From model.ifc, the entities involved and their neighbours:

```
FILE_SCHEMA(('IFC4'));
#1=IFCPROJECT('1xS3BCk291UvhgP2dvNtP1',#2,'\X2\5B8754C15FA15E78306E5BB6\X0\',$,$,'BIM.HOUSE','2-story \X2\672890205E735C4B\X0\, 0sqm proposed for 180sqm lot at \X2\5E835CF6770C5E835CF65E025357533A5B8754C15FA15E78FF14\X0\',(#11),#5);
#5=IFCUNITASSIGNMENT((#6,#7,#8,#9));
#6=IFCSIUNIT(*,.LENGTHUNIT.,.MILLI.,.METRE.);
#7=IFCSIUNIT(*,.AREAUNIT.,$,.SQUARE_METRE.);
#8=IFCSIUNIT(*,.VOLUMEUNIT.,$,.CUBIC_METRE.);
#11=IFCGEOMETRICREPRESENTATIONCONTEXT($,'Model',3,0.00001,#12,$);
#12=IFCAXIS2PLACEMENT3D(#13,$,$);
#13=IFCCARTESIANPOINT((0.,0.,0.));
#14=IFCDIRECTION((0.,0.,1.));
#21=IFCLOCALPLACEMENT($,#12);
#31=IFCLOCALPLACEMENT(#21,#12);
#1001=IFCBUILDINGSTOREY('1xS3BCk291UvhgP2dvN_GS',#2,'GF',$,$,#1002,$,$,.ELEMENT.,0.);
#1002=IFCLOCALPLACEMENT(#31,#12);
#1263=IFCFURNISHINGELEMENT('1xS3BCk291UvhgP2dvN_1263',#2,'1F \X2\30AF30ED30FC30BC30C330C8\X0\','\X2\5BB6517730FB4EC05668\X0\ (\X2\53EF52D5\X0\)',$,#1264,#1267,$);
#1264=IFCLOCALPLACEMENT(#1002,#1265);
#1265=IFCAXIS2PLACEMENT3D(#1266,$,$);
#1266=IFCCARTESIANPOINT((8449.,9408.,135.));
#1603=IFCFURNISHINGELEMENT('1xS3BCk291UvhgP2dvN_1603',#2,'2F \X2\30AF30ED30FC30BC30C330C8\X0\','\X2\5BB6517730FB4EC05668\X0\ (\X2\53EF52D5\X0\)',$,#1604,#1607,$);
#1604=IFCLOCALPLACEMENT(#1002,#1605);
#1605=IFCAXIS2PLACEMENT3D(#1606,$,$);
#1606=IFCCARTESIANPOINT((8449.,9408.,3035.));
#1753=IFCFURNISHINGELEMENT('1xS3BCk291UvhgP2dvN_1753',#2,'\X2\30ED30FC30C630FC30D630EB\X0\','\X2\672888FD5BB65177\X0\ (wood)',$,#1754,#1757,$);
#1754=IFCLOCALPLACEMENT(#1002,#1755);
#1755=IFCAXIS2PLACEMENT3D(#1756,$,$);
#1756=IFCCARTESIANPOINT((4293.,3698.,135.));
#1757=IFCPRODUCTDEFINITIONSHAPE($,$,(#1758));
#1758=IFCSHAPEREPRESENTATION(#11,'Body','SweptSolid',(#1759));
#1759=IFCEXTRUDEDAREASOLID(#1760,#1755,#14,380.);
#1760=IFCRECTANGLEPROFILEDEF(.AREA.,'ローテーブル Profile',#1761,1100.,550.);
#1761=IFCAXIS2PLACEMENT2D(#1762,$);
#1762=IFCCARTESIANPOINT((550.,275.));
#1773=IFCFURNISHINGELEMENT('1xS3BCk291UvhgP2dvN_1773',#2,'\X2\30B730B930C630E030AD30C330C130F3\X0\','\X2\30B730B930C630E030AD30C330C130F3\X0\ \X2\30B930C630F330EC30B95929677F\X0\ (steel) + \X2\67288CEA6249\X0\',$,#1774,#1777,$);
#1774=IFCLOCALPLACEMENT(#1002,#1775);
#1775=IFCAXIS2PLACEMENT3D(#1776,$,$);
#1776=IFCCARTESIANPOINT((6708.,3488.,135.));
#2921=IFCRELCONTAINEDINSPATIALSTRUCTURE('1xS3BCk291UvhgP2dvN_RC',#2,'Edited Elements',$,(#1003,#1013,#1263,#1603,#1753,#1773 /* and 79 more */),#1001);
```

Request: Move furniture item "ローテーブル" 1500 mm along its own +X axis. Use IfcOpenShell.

```python
import ifcopenshell
import ifcopenshell.api.geometry
import ifcopenshell.util.placement
import ifcopenshell.util.unit

model = ifcopenshell.open("model.ifc")
unit_scale = ifcopenshell.util.unit.calculate_unit_scale(model)

item = model.by_id(1753)
matrix = ifcopenshell.util.placement.get_local_placement(item.ObjectPlacement)
matrix[:3, 3] += matrix[:3, 0] * 1.5 / unit_scale
ifcopenshell.api.geometry.edit_object_placement(model, product=item, matrix=matrix, is_si=False)

print(ifcopenshell.util.placement.get_local_placement(item.ObjectPlacement).round(3) + 0.0)

model.write("model_v2.ifc")
```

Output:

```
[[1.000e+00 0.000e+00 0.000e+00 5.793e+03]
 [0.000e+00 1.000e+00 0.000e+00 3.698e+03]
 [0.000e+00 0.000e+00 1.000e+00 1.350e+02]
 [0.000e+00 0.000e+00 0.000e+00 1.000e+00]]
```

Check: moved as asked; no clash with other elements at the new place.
